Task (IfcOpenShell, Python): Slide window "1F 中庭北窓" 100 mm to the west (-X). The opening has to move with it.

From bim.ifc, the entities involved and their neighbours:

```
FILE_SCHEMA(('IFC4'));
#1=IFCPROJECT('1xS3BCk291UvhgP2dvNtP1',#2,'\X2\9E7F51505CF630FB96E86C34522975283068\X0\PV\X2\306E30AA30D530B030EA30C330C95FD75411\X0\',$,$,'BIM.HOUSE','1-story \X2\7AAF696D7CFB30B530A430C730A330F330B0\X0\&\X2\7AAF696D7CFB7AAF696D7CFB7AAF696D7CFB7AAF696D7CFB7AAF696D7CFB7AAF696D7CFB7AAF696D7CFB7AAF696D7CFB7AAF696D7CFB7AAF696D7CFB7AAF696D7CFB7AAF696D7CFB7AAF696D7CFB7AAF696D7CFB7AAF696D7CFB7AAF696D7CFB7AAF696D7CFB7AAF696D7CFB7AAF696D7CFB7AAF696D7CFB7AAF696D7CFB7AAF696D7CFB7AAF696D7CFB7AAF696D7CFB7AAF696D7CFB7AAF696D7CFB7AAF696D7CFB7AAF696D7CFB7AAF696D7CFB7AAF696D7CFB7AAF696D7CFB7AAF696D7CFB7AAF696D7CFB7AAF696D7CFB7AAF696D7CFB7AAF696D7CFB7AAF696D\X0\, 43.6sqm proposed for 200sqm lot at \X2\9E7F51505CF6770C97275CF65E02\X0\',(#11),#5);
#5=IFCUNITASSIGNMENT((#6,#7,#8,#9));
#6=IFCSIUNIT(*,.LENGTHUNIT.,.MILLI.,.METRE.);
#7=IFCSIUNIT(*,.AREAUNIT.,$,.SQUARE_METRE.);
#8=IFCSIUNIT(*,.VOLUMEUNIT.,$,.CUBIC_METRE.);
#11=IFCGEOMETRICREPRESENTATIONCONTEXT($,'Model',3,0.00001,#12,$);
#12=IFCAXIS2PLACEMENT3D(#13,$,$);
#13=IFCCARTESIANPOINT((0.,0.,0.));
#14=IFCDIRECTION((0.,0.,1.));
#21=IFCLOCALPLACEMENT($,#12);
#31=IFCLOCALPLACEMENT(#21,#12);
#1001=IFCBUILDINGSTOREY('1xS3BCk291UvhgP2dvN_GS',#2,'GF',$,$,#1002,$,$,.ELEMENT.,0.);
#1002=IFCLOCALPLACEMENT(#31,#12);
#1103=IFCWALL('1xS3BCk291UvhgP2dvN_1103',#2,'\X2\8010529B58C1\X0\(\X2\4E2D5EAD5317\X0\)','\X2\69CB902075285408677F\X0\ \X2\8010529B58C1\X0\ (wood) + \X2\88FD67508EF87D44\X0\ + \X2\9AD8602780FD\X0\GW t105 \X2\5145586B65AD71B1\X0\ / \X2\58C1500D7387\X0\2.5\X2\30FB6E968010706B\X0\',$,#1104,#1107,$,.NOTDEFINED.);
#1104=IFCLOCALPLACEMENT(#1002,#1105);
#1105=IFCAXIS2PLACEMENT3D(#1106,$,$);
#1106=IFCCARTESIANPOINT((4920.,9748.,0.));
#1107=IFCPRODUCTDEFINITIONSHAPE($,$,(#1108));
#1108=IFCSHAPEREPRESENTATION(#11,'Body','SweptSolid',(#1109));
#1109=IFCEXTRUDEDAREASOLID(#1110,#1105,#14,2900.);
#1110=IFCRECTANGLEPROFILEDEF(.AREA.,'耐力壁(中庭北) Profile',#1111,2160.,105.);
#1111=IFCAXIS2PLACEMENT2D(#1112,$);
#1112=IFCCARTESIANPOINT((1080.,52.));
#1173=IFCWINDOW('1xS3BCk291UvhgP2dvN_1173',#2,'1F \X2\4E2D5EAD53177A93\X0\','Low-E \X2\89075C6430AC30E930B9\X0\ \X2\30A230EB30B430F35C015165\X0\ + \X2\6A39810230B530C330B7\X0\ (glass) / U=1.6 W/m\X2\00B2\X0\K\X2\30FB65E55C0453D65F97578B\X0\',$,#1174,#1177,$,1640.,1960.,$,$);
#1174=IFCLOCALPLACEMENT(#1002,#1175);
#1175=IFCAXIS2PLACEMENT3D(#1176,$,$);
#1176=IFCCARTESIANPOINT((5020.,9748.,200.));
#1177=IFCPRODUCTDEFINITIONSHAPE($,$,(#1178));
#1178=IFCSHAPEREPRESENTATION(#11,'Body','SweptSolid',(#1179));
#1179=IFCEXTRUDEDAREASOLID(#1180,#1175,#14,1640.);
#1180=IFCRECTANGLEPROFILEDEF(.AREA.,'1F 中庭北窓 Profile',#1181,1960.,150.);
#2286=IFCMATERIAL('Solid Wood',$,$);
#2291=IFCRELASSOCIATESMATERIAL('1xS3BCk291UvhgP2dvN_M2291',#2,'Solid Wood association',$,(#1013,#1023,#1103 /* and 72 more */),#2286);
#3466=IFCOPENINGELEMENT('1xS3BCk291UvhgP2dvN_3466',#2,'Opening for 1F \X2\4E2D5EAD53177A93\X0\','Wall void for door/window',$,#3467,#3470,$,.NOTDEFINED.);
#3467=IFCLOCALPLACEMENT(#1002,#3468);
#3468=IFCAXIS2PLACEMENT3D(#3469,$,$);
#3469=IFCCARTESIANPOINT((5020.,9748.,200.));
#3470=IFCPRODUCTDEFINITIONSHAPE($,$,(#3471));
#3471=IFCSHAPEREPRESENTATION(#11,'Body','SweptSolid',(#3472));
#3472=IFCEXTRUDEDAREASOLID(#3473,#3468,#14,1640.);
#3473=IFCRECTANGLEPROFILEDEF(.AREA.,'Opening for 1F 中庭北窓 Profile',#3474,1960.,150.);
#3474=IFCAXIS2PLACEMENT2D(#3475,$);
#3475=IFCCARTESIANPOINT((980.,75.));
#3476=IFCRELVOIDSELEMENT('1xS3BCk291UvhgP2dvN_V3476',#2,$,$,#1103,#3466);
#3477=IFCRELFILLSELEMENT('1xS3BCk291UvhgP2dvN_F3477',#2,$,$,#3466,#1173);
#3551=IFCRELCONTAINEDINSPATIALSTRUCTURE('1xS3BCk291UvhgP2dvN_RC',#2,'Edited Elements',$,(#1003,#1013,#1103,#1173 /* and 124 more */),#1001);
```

```python
import ifcopenshell
import ifcopenshell.api.geometry
import ifcopenshell.util.placement
import ifcopenshell.util.unit

model = ifcopenshell.open("bim.ifc")
unit_scale = ifcopenshell.util.unit.calculate_unit_scale(model)

window = model.by_id(1173)
opening = window.FillsVoids[0].RelatingOpeningElement
wall = opening.VoidsElements[0].RelatingBuildingElement

wall_matrix = ifcopenshell.util.placement.get_local_placement(wall.ObjectPlacement)
shift = wall_matrix[:3, 0] * -0.1 / unit_scale
before = ifcopenshell.util.placement.get_local_placement(window.ObjectPlacement)[:3, 3].copy()

# The window is not placed relative to its opening, so move both.
for product in (opening, window):
    matrix = ifcopenshell.util.placement.get_local_placement(product.ObjectPlacement)
    matrix[:3, 3] += shift
    ifcopenshell.api.geometry.edit_object_placement(model, product=product, matrix=matrix, is_si=False)

after = ifcopenshell.util.placement.get_local_placement(window.ObjectPlacement)[:3, 3]
print("window moved by", (after - before).round(3) + 0.0)

model.write("bim_rev.ifc")
```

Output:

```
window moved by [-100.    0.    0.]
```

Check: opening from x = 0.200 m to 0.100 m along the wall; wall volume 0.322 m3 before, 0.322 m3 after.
